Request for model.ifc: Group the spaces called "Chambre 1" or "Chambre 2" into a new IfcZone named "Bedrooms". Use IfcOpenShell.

First a look at what the model holds.

```python
import ifcopenshell

model = ifcopenshell.open("model.ifc")
print(model.schema)
seen = {}
for space in model.by_type("IfcSpace"):
    seen[space.LongName] = seen.get(space.LongName, 0) + 1
for name, count in sorted(seen.items(), key=str):
    print(count, "x", name)
print("zones:", [z.Name for z in model.by_type("IfcZone")][:20])
```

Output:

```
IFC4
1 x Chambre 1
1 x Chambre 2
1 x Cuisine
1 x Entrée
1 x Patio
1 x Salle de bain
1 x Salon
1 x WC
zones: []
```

```python
import ifcopenshell
import ifcopenshell.api.group
import ifcopenshell.api.root

model = ifcopenshell.open("model.ifc")

names = {"Chambre 1", "Chambre 2"}
spaces = [s for s in model.by_type("IfcSpace") if s.LongName in names]

zone = ifcopenshell.api.root.create_entity(model, ifc_class="IfcZone", name="Bedrooms")
ifcopenshell.api.group.assign_group(model, products=spaces, group=zone)
print(len(spaces), "spaces in", zone.Name)

model.write("model_edited.ifc")
```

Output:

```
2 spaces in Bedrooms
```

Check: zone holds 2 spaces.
